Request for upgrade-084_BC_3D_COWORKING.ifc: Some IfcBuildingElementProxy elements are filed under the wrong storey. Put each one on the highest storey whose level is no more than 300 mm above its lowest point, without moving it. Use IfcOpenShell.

First a look at what the model holds.

```python
import ifcopenshell
import ifcopenshell.util.element
import ifcopenshell.util.placement

model = ifcopenshell.open("upgrade-084_BC_3D_COWORKING.ifc")
print(model.schema)
for storey in model.by_type("IfcBuildingStorey"):
    level = ifcopenshell.util.placement.get_storey_elevation(storey)
    count = sum(e.is_a("IfcBuildingElementProxy") for e in ifcopenshell.util.element.get_contained(storey))
    print(storey.id(), storey.Name, round(level, 3), count, sep=" | ")
```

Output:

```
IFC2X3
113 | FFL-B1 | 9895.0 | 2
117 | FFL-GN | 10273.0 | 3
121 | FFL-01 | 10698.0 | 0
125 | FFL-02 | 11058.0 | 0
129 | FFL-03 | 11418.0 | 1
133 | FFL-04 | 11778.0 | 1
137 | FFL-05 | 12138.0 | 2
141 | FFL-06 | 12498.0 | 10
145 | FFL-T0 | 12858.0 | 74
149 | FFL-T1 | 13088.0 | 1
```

```python
import ifcopenshell
import ifcopenshell.api.spatial
import ifcopenshell.geom
import ifcopenshell.util.element
import ifcopenshell.util.placement
import ifcopenshell.util.shape
import ifcopenshell.util.unit

model = ifcopenshell.open("upgrade-084_BC_3D_COWORKING.ifc")
unit_scale = ifcopenshell.util.unit.calculate_unit_scale(model)
settings = ifcopenshell.geom.settings()

levels = sorted(
    ((ifcopenshell.util.placement.get_storey_elevation(s) * unit_scale, s) for s in model.by_type("IfcBuildingStorey")),
    key=lambda pair: pair[0],
)

for e in model.by_type("IfcBuildingElementProxy"):
    current = e.ContainedInStructure[0].RelatingStructure if e.ContainedInStructure else None
    if current is None or not current.is_a("IfcBuildingStorey"):
        continue
    shape = ifcopenshell.geom.create_shape(settings, e)
    bottom = ifcopenshell.util.shape.get_shape_bottom_elevation(shape, shape.geometry)
    below = [s for level, s in levels if level <= bottom + 0.3]
    storey = below[-1] if below else levels[0][1]
    if storey != current:
        # assign_container keeps the world position.
        ifcopenshell.api.spatial.assign_container(model, products=[e], relating_structure=storey)
        print(e.id(), current.Name, "->", storey.Name)

model.write("upgrade-084_BC_3D_COWORKING_updated.ifc")
```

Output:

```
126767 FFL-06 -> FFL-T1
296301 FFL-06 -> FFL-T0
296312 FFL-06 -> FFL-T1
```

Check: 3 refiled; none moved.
